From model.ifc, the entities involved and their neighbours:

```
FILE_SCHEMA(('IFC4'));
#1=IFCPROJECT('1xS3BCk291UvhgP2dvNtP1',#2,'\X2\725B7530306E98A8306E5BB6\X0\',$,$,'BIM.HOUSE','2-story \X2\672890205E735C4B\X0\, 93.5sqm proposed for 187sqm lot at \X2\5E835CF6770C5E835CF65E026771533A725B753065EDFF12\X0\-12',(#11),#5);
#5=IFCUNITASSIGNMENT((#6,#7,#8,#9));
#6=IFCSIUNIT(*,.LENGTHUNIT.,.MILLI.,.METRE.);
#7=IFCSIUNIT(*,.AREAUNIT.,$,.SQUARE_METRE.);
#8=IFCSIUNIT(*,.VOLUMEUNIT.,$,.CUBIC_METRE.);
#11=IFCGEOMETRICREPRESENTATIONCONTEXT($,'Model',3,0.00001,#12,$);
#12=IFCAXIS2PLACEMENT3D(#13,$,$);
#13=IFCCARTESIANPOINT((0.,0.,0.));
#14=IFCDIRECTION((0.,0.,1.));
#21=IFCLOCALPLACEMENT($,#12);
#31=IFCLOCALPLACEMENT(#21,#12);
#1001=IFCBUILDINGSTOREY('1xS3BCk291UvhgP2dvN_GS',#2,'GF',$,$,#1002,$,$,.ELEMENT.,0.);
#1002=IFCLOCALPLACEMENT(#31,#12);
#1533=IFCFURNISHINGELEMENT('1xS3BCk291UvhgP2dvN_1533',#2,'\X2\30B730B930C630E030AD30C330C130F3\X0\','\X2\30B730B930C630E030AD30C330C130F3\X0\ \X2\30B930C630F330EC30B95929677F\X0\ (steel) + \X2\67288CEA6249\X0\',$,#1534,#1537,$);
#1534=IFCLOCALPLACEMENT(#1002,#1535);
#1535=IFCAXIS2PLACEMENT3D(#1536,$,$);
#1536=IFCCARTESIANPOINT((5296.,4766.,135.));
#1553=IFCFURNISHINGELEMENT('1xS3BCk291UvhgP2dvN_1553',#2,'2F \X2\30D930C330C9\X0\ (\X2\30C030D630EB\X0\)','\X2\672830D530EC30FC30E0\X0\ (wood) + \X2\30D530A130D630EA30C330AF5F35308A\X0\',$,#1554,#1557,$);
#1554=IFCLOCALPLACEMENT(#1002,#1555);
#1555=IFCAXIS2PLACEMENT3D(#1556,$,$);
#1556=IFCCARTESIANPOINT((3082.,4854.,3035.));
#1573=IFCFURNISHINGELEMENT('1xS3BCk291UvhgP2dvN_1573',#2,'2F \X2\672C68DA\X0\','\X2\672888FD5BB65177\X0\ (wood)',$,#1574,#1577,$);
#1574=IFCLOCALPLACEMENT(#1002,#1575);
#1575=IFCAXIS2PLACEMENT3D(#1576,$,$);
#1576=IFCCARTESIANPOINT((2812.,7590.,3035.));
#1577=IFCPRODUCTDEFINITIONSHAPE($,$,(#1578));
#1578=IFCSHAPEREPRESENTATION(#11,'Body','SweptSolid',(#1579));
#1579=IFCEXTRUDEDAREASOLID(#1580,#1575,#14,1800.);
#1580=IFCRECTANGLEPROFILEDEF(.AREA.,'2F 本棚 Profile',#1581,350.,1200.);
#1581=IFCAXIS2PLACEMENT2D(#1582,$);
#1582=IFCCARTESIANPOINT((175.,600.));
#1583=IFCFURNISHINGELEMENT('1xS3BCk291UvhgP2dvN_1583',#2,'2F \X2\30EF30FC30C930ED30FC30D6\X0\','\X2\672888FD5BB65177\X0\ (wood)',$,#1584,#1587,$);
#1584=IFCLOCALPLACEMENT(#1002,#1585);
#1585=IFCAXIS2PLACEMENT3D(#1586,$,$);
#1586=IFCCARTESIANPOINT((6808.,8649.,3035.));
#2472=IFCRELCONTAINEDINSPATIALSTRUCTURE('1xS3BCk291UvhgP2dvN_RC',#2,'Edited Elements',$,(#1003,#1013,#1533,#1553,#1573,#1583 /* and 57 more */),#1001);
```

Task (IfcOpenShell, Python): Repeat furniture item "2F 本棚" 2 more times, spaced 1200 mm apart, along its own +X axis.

```python
import ifcopenshell
import ifcopenshell.api.geometry
import ifcopenshell.api.root
import ifcopenshell.util.element
import ifcopenshell.util.placement
import ifcopenshell.util.unit

model = ifcopenshell.open("model.ifc")
unit_scale = ifcopenshell.util.unit.calculate_unit_scale(model)


def reuse_history(source, copy):
    """copy_class also copies each property set's owner history, people and application; keep the originals."""
    for rel in copy.IsDefinedBy:
        if rel.is_a("IfcRelDefinesByProperties") and (history := rel.RelatingPropertyDefinition.OwnerHistory):
            rel.RelatingPropertyDefinition.OwnerHistory = source.OwnerHistory
            ifcopenshell.util.element.remove_deep2(model, history)


source = model.by_id(1573)
base = ifcopenshell.util.placement.get_local_placement(source.ObjectPlacement)
step = base[:3, 0] * 1.2 / unit_scale

for i in range(1, 3):
    copy = ifcopenshell.api.root.copy_class(model, product=source)
    copy.Representation = ifcopenshell.util.element.copy_deep(
        model, source.Representation, exclude=["IfcGeometricRepresentationContext", "IfcRepresentationMap"]
    )
    reuse_history(source, copy)
    matrix = base.copy()
    matrix[:3, 3] += i * step
    print("added at", matrix[:3, 3].round(3) + 0.0)
    ifcopenshell.api.geometry.edit_object_placement(model, product=copy, matrix=matrix, is_si=False)

model.write("model_v2.ifc")
```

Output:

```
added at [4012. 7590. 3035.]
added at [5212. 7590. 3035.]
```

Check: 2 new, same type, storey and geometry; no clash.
